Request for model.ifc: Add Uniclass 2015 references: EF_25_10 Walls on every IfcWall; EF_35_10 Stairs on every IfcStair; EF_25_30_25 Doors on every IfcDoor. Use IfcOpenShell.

First a look at what the model holds.

```python
import ifcopenshell

model = ifcopenshell.open("model.ifc")
print(model.schema)
print("classifications:", [c.Name for c in model.by_type("IfcClassification")])
for ifc_class in ("IfcDoor", "IfcRoof", "IfcStair", "IfcWall", "IfcWindow"):
    print(ifc_class, len(model.by_type(ifc_class)))
```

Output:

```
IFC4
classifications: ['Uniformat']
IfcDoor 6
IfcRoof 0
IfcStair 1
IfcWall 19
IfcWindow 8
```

```python
import ifcopenshell
import ifcopenshell.api.classification

model = ifcopenshell.open("model.ifc")

system = ifcopenshell.api.classification.add_classification(model, classification="Uniclass 2015")

codes = {
    "IfcWall": ("EF_25_10", "Walls"),
    "IfcStair": ("EF_35_10", "Stairs"),
    "IfcDoor": ("EF_25_30_25", "Doors"),
}
for ifc_class, (code, name) in codes.items():
    products = model.by_type(ifc_class)
    ifcopenshell.api.classification.add_reference(
        model, products=products, classification=system, identification=code, name=name
    )
    print(code, len(products))

model.write("model-out.ifc")
```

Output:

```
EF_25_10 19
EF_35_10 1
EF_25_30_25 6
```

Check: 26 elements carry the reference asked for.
